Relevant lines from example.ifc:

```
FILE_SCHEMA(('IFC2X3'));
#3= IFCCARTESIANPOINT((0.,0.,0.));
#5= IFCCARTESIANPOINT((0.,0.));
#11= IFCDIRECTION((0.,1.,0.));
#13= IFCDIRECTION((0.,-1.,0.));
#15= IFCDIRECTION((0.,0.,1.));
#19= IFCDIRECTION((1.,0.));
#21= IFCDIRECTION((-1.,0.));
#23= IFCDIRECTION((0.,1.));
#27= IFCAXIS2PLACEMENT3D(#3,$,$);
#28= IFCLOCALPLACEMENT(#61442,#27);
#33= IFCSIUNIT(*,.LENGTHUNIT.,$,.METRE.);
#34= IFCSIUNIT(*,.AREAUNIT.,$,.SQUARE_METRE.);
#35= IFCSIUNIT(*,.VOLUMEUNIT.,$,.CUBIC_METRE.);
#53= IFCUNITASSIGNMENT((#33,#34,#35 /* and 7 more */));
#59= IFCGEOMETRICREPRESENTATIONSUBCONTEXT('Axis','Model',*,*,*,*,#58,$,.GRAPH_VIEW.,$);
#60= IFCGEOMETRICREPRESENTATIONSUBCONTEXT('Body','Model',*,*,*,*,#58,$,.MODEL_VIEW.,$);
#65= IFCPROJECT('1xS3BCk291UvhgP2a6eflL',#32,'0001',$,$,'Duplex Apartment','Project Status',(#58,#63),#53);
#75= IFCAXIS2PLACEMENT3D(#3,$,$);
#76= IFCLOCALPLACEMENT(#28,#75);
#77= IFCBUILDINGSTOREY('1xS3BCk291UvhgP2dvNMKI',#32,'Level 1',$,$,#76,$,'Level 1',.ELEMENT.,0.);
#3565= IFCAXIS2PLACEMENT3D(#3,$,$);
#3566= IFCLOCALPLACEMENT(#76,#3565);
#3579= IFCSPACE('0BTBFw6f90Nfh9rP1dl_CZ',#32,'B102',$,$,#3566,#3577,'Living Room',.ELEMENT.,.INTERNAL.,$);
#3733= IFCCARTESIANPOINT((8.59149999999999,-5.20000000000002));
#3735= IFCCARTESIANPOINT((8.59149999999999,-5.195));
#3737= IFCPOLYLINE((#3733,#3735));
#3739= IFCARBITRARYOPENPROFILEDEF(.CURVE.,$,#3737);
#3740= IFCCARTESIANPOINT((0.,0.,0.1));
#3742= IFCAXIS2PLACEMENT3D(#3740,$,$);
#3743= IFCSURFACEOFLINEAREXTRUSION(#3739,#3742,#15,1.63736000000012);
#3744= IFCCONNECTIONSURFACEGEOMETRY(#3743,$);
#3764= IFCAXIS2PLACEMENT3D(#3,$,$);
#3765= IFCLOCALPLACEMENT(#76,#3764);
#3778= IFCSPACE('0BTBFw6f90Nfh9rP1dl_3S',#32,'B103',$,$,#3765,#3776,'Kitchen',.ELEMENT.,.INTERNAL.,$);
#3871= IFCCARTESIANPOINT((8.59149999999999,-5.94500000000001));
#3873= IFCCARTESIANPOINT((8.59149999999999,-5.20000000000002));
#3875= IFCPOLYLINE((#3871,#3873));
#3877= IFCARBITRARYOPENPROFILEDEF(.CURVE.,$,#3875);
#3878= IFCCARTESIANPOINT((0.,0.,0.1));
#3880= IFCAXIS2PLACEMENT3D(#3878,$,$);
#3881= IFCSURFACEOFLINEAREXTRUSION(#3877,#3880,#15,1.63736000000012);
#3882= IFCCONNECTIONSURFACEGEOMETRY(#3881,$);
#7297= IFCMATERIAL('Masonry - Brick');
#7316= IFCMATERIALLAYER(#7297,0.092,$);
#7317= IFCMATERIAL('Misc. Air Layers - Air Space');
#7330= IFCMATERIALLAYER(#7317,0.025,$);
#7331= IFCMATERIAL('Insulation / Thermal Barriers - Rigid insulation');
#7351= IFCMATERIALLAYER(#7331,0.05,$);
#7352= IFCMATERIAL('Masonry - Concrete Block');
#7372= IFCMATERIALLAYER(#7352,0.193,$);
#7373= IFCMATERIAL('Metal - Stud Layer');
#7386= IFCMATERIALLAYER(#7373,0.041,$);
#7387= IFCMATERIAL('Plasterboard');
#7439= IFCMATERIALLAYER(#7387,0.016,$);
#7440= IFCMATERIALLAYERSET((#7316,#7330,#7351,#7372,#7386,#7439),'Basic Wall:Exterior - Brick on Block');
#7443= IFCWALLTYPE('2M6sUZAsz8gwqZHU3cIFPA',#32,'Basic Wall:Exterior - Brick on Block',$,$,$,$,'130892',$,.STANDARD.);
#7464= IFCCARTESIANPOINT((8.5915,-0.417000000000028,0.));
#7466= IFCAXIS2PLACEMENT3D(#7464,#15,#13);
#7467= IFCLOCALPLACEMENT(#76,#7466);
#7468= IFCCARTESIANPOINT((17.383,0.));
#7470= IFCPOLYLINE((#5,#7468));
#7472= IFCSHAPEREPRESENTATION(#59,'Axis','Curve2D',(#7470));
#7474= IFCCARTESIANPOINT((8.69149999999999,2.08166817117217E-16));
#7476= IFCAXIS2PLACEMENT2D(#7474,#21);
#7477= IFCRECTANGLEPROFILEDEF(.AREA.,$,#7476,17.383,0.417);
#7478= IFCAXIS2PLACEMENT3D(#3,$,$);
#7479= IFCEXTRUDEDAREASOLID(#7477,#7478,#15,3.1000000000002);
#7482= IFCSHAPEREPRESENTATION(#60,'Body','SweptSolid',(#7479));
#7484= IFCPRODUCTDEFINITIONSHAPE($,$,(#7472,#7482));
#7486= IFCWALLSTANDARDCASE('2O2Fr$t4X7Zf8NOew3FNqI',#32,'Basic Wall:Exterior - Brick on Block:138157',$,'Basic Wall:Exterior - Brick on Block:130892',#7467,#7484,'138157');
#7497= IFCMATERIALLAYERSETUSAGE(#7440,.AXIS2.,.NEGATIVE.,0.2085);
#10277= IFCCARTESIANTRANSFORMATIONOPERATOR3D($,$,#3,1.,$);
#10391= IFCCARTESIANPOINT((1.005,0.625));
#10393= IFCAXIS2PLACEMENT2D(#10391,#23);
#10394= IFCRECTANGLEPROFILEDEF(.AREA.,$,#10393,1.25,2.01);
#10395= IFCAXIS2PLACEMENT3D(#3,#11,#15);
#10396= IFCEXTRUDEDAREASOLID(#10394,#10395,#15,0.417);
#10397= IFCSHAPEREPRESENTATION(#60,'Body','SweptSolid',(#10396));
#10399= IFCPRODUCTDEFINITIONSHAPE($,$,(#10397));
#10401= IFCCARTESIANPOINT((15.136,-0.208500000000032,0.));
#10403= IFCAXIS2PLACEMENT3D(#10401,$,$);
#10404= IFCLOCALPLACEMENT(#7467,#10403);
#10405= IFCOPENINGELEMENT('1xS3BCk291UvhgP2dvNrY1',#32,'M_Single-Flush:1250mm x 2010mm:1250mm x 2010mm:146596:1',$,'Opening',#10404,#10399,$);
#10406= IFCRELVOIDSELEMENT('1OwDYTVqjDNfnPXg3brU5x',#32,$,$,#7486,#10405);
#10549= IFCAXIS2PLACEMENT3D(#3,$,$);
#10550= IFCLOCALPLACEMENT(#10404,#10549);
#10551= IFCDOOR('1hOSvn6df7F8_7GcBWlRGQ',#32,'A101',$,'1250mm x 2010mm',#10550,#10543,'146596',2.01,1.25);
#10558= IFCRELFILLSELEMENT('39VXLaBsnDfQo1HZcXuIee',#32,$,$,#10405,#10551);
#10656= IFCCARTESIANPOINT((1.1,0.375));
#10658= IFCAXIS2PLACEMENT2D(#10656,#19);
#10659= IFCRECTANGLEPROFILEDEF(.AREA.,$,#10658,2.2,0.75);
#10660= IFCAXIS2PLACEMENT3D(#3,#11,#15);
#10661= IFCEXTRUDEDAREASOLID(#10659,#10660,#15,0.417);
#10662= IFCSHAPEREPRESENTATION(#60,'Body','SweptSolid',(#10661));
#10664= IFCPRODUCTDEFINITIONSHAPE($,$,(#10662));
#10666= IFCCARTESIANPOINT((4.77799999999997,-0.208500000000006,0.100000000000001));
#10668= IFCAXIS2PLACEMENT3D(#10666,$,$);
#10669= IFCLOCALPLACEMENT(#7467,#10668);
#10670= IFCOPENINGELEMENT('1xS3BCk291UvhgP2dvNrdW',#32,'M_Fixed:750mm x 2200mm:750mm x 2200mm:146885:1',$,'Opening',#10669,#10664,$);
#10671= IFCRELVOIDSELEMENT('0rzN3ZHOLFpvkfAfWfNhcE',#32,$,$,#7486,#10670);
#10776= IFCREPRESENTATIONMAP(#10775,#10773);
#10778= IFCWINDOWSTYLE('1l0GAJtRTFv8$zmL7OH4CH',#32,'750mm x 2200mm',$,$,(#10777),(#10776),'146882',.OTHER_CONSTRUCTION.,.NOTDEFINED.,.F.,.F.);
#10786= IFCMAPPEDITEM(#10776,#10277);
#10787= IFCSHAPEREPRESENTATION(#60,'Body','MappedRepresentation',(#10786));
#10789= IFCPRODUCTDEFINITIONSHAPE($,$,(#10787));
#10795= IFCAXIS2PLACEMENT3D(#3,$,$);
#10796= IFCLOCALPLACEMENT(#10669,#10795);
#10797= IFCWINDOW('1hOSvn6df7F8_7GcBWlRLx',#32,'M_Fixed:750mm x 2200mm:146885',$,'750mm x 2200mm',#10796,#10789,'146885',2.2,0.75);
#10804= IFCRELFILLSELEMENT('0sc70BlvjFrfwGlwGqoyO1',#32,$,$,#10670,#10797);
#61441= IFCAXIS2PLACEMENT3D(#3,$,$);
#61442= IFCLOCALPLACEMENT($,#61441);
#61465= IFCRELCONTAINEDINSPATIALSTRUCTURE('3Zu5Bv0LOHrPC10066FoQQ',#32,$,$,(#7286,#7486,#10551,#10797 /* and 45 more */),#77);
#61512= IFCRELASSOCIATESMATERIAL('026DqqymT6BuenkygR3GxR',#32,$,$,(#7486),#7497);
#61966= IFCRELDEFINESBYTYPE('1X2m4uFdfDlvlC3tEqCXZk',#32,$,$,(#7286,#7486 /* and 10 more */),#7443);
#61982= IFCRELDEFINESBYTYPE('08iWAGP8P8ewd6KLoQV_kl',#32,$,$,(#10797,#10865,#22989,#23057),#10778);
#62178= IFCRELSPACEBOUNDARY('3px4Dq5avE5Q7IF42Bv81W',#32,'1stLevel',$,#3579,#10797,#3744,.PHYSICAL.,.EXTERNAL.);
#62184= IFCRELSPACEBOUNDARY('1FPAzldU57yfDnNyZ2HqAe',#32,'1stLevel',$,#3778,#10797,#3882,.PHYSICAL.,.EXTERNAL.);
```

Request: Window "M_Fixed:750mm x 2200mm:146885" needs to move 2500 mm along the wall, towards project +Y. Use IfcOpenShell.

```python
import numpy as np
import ifcopenshell
import ifcopenshell.api.geometry
import ifcopenshell.util.placement
import ifcopenshell.util.unit

model = ifcopenshell.open("example.ifc")
unit_scale = ifcopenshell.util.unit.calculate_unit_scale(model)

window = model.by_guid("1hOSvn6df7F8_7GcBWlRLx")
opening = window.FillsVoids[0].RelatingOpeningElement
wall = opening.VoidsElements[0].RelatingBuildingElement

wall_matrix = ifcopenshell.util.placement.get_local_placement(wall.ObjectPlacement)
shift = wall_matrix[:3, 0] * -2.5 / unit_scale
before = ifcopenshell.util.placement.get_local_placement(window.ObjectPlacement)[:3, 3].copy()

# The window is placed relative to its opening, so it follows when the opening moves.
matrix = ifcopenshell.util.placement.get_local_placement(opening.ObjectPlacement)
matrix[:3, 3] += shift
ifcopenshell.api.geometry.edit_object_placement(
    model, product=opening, matrix=matrix, is_si=False, should_transform_children=True
)

# Space boundary surfaces are stored in each space's coordinates; move them too.
for rel in window.ProvidesBoundaries:
    if not rel.ConnectionGeometry:
        continue
    surface = rel.ConnectionGeometry.SurfaceOnRelatingElement
    space_matrix = ifcopenshell.util.placement.get_local_placement(rel.RelatingSpace.ObjectPlacement)
    point = np.array(surface.Position.Location.Coordinates) + space_matrix[:3, :3].T @ shift
    surface.Position = model.createIfcAxis2Placement3D(
        model.createIfcCartesianPoint(point.tolist()), surface.Position.Axis, surface.Position.RefDirection
    )

after = ifcopenshell.util.placement.get_local_placement(window.ObjectPlacement)[:3, 3]
print("window moved by", (after - before).round(3) + 0.0)

model.write("example_v2.ifc")
```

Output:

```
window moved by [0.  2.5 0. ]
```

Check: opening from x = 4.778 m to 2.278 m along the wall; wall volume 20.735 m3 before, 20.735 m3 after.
